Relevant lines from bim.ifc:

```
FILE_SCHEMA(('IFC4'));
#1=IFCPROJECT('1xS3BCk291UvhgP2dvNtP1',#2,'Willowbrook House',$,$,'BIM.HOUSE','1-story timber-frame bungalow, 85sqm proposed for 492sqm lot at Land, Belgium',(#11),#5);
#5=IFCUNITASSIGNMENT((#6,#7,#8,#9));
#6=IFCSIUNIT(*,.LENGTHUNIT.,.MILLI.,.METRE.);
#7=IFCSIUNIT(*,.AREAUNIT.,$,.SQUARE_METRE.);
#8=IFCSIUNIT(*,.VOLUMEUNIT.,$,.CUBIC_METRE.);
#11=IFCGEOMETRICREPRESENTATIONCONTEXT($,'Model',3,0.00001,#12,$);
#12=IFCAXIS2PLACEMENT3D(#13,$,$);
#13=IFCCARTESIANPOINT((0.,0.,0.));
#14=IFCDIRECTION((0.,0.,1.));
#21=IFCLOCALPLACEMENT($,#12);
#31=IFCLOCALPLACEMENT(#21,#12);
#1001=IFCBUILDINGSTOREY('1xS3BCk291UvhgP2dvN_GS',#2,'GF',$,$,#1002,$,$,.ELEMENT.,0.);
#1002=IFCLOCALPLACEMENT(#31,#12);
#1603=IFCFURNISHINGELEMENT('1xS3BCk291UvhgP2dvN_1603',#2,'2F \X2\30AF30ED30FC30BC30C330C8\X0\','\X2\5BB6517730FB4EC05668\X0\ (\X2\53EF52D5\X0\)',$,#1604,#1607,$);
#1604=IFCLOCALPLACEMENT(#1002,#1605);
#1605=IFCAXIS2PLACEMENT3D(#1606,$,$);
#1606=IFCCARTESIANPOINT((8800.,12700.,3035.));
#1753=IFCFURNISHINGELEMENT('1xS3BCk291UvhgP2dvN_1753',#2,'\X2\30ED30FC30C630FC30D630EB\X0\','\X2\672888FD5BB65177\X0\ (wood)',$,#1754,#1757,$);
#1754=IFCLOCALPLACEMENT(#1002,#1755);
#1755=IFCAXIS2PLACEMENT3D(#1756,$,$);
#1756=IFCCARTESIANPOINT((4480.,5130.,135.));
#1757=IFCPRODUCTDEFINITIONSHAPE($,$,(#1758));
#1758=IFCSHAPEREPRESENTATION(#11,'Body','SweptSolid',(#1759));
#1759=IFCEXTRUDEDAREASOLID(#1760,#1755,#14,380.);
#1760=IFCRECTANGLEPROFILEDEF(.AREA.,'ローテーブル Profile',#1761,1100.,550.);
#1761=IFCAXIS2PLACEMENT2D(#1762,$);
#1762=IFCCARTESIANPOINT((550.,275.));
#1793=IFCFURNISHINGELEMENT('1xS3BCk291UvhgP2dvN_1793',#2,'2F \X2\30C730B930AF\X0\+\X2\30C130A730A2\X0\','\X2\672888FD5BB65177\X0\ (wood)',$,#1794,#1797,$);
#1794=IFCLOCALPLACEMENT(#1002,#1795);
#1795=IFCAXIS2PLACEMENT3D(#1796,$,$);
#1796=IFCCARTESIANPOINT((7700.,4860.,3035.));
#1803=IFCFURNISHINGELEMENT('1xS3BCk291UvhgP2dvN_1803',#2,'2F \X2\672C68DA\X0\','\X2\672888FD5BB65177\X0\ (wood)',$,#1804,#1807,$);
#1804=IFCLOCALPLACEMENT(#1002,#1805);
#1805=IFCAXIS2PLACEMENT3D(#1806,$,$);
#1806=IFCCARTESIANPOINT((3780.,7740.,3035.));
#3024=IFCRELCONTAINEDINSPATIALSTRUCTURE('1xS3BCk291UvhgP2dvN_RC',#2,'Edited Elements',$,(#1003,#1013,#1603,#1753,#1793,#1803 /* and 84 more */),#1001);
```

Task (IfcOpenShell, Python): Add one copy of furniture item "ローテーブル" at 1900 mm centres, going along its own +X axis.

```python
import ifcopenshell
import ifcopenshell.api.geometry
import ifcopenshell.api.root
import ifcopenshell.util.element
import ifcopenshell.util.placement
import ifcopenshell.util.unit

model = ifcopenshell.open("bim.ifc")
unit_scale = ifcopenshell.util.unit.calculate_unit_scale(model)


def reuse_history(source, copy):
    """copy_class also copies each property set's owner history, people and application; keep the originals."""
    for rel in copy.IsDefinedBy:
        if rel.is_a("IfcRelDefinesByProperties") and (history := rel.RelatingPropertyDefinition.OwnerHistory):
            rel.RelatingPropertyDefinition.OwnerHistory = source.OwnerHistory
            ifcopenshell.util.element.remove_deep2(model, history)


source = model.by_guid("1xS3BCk291UvhgP2dvN_1753")
base = ifcopenshell.util.placement.get_local_placement(source.ObjectPlacement)
step = base[:3, 0] * 1.9 / unit_scale

for i in range(1, 2):
    copy = ifcopenshell.api.root.copy_class(model, product=source)
    copy.Representation = ifcopenshell.util.element.copy_deep(
        model, source.Representation, exclude=["IfcGeometricRepresentationContext", "IfcRepresentationMap"]
    )
    reuse_history(source, copy)
    matrix = base.copy()
    matrix[:3, 3] += i * step
    print("added at", matrix[:3, 3].round(3) + 0.0)
    ifcopenshell.api.geometry.edit_object_placement(model, product=copy, matrix=matrix, is_si=False)

model.write("bim_edited.ifc")
```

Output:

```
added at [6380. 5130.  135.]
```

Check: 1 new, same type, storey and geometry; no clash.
